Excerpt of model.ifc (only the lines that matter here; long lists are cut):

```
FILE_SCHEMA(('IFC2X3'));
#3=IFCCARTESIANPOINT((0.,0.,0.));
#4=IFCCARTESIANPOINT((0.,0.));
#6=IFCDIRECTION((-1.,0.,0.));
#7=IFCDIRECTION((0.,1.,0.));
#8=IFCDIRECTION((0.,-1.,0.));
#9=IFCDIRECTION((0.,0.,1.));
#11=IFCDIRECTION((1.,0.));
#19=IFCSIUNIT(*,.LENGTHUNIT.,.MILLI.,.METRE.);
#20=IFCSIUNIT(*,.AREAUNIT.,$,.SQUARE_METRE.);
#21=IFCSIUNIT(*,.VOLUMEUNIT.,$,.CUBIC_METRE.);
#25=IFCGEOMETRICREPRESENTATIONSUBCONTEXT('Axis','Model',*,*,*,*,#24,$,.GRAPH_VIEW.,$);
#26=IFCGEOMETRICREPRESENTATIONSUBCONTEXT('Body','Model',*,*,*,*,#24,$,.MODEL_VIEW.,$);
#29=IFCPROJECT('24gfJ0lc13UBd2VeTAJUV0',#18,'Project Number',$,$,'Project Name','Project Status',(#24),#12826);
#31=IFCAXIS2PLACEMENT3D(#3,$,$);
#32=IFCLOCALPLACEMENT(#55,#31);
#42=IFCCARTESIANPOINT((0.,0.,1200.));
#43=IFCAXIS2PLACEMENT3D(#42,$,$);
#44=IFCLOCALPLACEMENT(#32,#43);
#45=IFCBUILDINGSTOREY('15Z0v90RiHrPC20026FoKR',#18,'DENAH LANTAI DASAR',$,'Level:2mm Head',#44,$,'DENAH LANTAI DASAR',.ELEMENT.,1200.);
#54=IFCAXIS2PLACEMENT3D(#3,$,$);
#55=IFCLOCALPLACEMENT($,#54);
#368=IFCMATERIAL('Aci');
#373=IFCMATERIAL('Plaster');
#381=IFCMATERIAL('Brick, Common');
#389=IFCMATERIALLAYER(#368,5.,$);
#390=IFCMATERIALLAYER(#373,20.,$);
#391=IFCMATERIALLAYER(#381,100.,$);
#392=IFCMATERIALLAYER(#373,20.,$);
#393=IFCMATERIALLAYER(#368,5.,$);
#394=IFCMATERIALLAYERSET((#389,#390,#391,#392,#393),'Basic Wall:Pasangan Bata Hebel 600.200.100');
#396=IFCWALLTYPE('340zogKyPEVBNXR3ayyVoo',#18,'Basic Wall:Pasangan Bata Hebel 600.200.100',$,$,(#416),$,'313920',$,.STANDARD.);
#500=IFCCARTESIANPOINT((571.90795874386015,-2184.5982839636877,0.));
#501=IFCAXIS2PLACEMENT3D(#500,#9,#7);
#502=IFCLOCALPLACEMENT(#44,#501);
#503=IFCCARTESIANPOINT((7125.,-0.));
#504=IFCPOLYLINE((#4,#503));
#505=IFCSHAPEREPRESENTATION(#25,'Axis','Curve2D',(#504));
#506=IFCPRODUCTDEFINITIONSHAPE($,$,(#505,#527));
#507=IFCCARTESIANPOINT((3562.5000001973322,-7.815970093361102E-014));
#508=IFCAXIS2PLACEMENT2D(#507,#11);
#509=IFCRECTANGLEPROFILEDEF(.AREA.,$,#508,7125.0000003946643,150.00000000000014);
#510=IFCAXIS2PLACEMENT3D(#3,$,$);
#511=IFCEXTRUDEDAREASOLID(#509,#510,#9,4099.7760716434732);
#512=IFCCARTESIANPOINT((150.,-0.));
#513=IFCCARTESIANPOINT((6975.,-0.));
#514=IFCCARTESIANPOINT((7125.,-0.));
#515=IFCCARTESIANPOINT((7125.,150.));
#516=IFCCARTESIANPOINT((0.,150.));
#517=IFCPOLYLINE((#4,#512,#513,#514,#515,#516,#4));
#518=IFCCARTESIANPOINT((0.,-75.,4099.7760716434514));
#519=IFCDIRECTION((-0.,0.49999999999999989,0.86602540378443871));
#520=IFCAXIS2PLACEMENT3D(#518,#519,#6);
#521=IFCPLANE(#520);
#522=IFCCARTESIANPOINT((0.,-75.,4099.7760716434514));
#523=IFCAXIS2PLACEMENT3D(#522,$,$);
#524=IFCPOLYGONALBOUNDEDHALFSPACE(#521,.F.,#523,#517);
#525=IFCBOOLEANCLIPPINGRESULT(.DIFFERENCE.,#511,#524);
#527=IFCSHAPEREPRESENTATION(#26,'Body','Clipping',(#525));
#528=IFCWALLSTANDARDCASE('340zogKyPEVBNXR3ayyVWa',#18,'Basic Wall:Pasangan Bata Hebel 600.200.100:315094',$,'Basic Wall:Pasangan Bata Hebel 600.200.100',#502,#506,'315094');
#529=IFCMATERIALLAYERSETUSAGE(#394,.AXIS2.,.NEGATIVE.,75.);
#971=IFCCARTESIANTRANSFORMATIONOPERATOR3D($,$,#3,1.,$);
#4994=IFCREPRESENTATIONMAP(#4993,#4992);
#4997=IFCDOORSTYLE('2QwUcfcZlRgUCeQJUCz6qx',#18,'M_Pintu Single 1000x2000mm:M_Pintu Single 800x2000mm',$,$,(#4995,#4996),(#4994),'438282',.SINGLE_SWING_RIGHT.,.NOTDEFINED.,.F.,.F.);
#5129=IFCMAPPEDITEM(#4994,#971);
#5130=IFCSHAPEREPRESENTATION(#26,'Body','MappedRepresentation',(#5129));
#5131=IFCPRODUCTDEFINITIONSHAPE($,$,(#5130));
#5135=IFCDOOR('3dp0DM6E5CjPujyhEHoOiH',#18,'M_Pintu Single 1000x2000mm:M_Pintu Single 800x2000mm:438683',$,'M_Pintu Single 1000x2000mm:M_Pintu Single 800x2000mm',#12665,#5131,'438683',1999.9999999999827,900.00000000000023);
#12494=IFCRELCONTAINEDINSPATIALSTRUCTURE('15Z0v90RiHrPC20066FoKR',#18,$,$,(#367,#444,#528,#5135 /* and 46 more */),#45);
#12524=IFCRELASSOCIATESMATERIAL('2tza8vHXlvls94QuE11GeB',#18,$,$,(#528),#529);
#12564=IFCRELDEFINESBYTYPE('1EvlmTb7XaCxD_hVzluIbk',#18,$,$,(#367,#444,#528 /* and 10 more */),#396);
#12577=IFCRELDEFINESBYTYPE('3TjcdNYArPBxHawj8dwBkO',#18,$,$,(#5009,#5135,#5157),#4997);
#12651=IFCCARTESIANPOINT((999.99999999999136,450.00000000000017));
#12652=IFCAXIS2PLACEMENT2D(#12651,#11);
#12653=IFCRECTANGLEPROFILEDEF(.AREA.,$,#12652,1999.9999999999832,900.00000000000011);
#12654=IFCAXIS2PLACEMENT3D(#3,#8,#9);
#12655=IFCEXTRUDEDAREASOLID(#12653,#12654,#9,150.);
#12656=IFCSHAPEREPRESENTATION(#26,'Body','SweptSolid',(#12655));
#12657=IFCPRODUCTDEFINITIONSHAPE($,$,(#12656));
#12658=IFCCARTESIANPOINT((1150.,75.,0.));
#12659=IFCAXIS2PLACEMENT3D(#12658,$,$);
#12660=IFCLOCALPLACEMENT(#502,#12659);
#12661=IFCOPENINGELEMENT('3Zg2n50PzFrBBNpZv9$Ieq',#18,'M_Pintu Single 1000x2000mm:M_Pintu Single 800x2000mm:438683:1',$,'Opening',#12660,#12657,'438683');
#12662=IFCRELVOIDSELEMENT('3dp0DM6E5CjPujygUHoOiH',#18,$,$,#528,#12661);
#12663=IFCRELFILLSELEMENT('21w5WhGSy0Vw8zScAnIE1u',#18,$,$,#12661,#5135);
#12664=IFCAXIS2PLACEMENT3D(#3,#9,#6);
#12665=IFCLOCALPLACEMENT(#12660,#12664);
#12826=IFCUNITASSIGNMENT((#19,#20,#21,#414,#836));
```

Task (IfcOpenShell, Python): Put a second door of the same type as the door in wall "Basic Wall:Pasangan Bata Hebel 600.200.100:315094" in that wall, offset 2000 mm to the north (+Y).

```python
import ifcopenshell
import ifcopenshell.api.feature
import ifcopenshell.api.geometry
import ifcopenshell.api.root
import ifcopenshell.geom
import ifcopenshell.util.element
import ifcopenshell.util.placement
import ifcopenshell.util.shape
import ifcopenshell.util.unit

model = ifcopenshell.open("model.ifc")
unit_scale = ifcopenshell.util.unit.calculate_unit_scale(model)
settings = ifcopenshell.geom.settings()


def volume(element):
    """Net volume in cubic metres, openings subtracted."""
    shape = ifcopenshell.geom.create_shape(settings, element)
    return ifcopenshell.util.shape.get_volume(shape.geometry)


def reuse_history(source, copy):
    """copy_class also copies each property set's owner history, people and application; keep the originals."""
    for rel in copy.IsDefinedBy:
        if rel.is_a("IfcRelDefinesByProperties") and (history := rel.RelatingPropertyDefinition.OwnerHistory):
            rel.RelatingPropertyDefinition.OwnerHistory = source.OwnerHistory
            ifcopenshell.util.element.remove_deep2(model, history)


door = model.by_id(5135)
opening = door.FillsVoids[0].RelatingOpeningElement
wall = opening.VoidsElements[0].RelatingBuildingElement
before = volume(wall)
shift = ifcopenshell.util.placement.get_local_placement(wall.ObjectPlacement)[:3, 0] * 2 / unit_scale

# copy_class copies the void relationship, type, container and properties, but no geometry.
new_opening = ifcopenshell.api.root.copy_class(model, product=opening)
new_opening.Representation = ifcopenshell.util.element.copy_deep(
    model, opening.Representation, exclude=["IfcGeometricRepresentationContext", "IfcRepresentationMap"]
)
new_opening.Name = "M_Pintu Single 1000x2000mm:M_Pintu Single 800x2000mm"
new_opening.Tag = None
new_door = ifcopenshell.api.root.copy_class(model, product=door)
new_door.Representation = ifcopenshell.util.element.copy_deep(
    model, door.Representation, exclude=["IfcGeometricRepresentationContext", "IfcRepresentationMap"]
)
new_door.Name = "M_Pintu Single 1000x2000mm:M_Pintu Single 800x2000mm"
new_door.Tag = None
reuse_history(door, new_door)
fills = ifcopenshell.api.feature.add_filling(model, opening=new_opening, element=new_door)
fills.OwnerHistory = new_door.OwnerHistory  # required in IFC2X3

for old, new in ((opening, new_opening), (door, new_door)):
    matrix = ifcopenshell.util.placement.get_local_placement(old.ObjectPlacement)
    matrix[:3, 3] += shift
    ifcopenshell.api.geometry.edit_object_placement(model, product=new, matrix=matrix, is_si=False)

after = volume(wall)

print(f"wall volume {before:.3f} -> {after:.3f} m3")

model.write("model_updated.ifc")
```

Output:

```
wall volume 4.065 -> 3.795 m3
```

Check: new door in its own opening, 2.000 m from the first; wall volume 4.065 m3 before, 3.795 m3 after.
